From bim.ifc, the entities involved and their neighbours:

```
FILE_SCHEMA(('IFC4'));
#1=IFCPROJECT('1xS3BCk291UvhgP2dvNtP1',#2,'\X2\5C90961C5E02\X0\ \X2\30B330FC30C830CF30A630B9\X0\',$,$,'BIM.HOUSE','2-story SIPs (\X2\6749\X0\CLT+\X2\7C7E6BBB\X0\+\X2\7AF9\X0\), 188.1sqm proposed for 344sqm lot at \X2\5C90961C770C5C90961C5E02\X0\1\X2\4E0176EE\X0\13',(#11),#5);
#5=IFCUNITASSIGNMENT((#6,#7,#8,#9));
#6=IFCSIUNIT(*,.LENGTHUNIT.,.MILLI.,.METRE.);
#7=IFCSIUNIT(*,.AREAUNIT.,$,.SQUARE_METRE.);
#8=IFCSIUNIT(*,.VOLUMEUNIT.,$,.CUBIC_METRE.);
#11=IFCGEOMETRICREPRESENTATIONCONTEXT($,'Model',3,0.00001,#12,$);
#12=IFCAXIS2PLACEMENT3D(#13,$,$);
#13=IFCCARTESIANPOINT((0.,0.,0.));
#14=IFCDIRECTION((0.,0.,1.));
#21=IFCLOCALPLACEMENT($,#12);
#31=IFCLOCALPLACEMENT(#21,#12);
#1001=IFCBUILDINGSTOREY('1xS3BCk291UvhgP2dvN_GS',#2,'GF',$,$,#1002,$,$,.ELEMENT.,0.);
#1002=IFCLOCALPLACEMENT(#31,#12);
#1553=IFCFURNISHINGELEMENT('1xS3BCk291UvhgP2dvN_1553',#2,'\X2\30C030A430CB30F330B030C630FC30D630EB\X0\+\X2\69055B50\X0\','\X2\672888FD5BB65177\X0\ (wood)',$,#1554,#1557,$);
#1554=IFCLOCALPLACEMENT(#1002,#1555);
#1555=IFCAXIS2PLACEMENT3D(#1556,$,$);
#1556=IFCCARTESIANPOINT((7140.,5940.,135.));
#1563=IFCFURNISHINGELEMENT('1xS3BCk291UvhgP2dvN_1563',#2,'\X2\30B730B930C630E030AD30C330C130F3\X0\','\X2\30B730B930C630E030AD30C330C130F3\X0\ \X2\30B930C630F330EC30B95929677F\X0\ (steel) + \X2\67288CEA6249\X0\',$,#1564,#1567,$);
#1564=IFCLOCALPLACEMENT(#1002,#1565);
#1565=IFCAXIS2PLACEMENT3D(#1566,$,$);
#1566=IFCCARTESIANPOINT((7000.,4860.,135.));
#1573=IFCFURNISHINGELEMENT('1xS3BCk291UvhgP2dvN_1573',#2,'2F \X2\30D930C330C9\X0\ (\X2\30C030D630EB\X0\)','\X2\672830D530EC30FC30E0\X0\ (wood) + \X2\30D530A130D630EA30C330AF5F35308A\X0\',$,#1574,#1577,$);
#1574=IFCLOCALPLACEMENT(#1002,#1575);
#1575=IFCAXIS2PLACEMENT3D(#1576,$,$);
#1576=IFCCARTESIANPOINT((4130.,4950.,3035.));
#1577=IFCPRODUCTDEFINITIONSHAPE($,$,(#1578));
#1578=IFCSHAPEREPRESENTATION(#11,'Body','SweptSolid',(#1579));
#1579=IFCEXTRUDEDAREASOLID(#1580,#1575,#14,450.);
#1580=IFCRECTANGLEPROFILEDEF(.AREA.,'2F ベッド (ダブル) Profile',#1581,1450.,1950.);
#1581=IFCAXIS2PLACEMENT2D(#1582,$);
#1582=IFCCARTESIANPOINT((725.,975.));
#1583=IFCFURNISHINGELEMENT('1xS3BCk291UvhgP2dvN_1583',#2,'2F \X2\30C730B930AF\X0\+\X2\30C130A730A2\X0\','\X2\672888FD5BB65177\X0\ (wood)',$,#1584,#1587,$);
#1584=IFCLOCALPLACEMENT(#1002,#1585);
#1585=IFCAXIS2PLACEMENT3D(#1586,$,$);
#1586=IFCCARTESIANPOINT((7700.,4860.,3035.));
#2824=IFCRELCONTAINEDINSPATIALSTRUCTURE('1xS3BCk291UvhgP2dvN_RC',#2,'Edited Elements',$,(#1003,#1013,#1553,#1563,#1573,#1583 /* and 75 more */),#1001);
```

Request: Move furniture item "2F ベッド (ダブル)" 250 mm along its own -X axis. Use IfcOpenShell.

```python
import ifcopenshell
import ifcopenshell.api.geometry
import ifcopenshell.util.placement
import ifcopenshell.util.unit

model = ifcopenshell.open("bim.ifc")
unit_scale = ifcopenshell.util.unit.calculate_unit_scale(model)

item = model.by_id(1573)
matrix = ifcopenshell.util.placement.get_local_placement(item.ObjectPlacement)
matrix[:3, 3] -= matrix[:3, 0] * 0.25 / unit_scale
ifcopenshell.api.geometry.edit_object_placement(model, product=item, matrix=matrix, is_si=False)

print(ifcopenshell.util.placement.get_local_placement(item.ObjectPlacement).round(3) + 0.0)

model.write("bim-out.ifc")
```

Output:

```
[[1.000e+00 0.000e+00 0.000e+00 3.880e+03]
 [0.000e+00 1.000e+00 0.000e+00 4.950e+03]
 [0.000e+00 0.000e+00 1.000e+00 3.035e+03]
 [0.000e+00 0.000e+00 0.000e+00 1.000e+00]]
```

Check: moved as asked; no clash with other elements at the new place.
